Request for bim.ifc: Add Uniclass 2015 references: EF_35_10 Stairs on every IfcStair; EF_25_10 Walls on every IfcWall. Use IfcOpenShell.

First a look at what the model holds.

```python
import ifcopenshell

model = ifcopenshell.open("bim.ifc")
print(model.schema)
print("classifications:", [c.Name for c in model.by_type("IfcClassification")])
for ifc_class in ("IfcDoor", "IfcRoof", "IfcStair", "IfcWall", "IfcWindow"):
    print(ifc_class, len(model.by_type(ifc_class)))
```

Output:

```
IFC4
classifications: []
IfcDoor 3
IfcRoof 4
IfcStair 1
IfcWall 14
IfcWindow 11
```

```python
import ifcopenshell
import ifcopenshell.api.classification

model = ifcopenshell.open("bim.ifc")

system = ifcopenshell.api.classification.add_classification(model, classification="Uniclass 2015")

codes = {
    "IfcStair": ("EF_35_10", "Stairs"),
    "IfcWall": ("EF_25_10", "Walls"),
}
for ifc_class, (code, name) in codes.items():
    products = model.by_type(ifc_class)
    ifcopenshell.api.classification.add_reference(
        model, products=products, classification=system, identification=code, name=name
    )
    print(code, len(products))

model.write("bim-out.ifc")
```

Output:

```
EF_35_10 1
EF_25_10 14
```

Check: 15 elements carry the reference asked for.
